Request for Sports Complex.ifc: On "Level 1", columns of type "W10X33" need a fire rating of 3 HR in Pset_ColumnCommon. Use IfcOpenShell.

First a look at what the model holds.

```python
import ifcopenshell
import ifcopenshell.util.element

model = ifcopenshell.open("Sports Complex.ifc")
print(model.schema)
storey = next(s for s in model.by_type("IfcBuildingStorey") if s.Name == "Level 1")
columns = [e for e in ifcopenshell.util.element.get_decomposition(storey) if e.is_a("IfcColumn")]
seen = {}
for e in columns:
    element_type = ifcopenshell.util.element.get_type(e)
    key = (element_type.Name if element_type != e and element_type else None, ifcopenshell.util.element.get_pset(e, "Pset_ColumnCommon", "FireRating"))
    seen[key] = seen.get(key, 0) + 1
for (name, value), count in sorted(seen.items(), key=str):
    print(count, "x", name, "|", value)
```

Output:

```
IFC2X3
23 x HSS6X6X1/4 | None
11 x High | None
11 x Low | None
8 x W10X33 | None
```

```python
import ifcopenshell
import ifcopenshell.api.pset
import ifcopenshell.util.element

model = ifcopenshell.open("Sports Complex.ifc")

storey = next(s for s in model.by_type("IfcBuildingStorey") if s.Name == "Level 1")
columns = [e for e in ifcopenshell.util.element.get_decomposition(storey) if e.is_a("IfcColumn")]

count = 0
for e in columns:
    element_type = ifcopenshell.util.element.get_type(e)
    if element_type in (None, e) or element_type.Name != "W10X33":
        continue
    # add_pset returns the element's existing set when there is one.
    pset = ifcopenshell.api.pset.add_pset(model, product=e, name="Pset_ColumnCommon")
    ifcopenshell.api.pset.edit_pset(model, pset=pset, properties={"FireRating": "3 HR"})
    count += 1

print(count, "columns updated")

model.write("Sports Complex_updated.ifc")
```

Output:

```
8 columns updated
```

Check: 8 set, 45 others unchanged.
